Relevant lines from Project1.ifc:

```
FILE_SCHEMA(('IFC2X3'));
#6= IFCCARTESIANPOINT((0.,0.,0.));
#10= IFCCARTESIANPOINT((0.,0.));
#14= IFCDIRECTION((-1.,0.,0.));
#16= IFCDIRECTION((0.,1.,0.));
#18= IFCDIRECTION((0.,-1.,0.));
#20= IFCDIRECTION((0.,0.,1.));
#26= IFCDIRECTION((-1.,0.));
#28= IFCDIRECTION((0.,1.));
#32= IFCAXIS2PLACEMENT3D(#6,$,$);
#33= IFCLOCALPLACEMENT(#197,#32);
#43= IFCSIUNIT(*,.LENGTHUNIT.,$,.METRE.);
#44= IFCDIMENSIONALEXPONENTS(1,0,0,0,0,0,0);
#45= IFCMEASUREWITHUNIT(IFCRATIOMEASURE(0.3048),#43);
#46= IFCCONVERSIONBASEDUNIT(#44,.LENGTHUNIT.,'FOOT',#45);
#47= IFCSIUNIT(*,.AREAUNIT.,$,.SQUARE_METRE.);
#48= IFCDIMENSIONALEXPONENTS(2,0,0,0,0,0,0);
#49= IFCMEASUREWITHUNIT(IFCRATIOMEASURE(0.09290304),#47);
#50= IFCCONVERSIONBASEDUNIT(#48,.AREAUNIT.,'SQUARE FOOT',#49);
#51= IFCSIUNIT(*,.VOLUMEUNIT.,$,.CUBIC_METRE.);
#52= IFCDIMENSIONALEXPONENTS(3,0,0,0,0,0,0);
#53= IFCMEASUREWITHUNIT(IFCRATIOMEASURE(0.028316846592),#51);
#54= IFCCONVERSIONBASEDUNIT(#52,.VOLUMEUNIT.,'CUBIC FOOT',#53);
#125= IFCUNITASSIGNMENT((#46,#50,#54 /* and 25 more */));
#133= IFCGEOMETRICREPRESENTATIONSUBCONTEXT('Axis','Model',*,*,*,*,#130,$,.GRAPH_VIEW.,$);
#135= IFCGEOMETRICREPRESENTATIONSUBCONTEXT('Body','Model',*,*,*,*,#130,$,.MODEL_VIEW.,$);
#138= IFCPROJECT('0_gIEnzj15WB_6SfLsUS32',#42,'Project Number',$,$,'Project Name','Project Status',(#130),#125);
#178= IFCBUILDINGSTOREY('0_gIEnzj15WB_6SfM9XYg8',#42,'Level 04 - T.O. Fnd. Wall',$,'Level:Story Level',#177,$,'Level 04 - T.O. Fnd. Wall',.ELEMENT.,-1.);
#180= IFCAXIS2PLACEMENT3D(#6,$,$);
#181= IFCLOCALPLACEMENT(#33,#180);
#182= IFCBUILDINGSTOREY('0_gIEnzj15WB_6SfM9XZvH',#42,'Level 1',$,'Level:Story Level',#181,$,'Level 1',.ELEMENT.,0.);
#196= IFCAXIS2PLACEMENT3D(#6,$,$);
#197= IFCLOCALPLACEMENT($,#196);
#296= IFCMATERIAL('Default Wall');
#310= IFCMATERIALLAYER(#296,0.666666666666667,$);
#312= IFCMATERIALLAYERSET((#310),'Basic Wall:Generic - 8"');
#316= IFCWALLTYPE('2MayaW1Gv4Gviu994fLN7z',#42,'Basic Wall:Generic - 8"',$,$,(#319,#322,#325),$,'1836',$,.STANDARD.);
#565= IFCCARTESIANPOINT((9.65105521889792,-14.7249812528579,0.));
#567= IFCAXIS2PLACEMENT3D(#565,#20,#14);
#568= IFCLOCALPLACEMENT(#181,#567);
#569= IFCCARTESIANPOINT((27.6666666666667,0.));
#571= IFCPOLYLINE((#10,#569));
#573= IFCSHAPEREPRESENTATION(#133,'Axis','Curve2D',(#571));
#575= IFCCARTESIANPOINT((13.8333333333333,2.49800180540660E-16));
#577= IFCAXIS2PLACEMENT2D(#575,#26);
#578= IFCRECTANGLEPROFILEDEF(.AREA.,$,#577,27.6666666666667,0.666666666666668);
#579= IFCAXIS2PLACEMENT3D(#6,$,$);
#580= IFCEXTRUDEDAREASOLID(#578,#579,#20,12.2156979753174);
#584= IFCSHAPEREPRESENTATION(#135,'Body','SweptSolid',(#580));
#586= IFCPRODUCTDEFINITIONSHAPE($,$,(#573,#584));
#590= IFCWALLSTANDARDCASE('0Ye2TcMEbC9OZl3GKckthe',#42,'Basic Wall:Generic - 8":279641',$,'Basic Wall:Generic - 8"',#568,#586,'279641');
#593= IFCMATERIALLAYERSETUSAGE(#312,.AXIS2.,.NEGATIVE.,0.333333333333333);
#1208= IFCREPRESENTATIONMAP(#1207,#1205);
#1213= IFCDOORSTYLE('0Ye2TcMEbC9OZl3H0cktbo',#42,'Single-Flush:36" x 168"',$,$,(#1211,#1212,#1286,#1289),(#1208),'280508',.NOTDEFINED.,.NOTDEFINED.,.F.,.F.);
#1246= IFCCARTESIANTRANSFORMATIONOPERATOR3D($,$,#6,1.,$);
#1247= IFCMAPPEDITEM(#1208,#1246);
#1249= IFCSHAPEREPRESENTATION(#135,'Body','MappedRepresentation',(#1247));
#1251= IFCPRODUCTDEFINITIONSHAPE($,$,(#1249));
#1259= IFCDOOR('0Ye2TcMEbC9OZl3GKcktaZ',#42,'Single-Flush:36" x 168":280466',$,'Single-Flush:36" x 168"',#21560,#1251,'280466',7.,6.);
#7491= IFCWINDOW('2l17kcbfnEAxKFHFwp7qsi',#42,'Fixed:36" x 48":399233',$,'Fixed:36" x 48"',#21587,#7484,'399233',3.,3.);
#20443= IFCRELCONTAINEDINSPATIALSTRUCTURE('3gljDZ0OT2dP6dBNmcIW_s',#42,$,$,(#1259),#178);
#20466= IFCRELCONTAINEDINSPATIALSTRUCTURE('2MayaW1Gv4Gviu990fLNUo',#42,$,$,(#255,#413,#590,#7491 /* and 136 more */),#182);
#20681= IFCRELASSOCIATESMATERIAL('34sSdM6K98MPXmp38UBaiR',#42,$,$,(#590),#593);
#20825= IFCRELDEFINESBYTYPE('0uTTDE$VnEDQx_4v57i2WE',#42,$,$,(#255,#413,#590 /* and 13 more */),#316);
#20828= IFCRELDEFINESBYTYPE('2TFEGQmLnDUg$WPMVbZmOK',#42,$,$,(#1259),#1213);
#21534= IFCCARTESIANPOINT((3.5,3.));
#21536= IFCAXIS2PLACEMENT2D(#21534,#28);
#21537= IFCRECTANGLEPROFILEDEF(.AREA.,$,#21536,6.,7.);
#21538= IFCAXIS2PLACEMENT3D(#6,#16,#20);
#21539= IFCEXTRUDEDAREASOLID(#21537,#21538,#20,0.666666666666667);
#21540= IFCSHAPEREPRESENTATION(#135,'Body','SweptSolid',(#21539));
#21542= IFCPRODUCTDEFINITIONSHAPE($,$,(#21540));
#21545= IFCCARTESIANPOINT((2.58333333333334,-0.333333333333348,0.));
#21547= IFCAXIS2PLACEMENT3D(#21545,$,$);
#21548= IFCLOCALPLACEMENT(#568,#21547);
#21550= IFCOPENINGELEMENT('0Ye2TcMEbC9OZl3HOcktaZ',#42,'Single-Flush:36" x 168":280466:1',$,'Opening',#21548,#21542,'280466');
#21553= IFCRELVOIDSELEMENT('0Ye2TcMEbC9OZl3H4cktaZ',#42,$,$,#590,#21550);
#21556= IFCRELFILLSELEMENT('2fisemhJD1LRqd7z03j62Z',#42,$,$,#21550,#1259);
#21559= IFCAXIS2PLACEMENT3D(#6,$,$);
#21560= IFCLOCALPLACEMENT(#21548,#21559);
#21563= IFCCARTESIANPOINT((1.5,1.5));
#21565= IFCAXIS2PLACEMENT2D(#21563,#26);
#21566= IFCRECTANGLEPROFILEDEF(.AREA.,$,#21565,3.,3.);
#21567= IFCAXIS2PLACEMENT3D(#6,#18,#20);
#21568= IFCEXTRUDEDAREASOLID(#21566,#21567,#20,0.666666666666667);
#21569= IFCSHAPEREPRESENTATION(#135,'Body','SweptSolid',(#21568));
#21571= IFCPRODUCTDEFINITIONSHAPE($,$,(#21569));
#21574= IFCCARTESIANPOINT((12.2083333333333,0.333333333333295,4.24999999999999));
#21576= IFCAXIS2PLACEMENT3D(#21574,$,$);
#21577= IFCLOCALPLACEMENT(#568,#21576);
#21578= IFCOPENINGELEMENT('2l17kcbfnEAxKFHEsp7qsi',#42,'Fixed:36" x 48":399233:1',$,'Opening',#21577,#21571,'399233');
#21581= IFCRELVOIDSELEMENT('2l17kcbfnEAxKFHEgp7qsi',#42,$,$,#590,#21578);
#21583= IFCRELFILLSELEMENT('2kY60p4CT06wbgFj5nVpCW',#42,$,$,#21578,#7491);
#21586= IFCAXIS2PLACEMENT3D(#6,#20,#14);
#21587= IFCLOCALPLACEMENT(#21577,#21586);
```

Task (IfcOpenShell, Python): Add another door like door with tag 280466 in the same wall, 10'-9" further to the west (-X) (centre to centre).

```python
import ifcopenshell
import ifcopenshell.api.feature
import ifcopenshell.api.geometry
import ifcopenshell.api.root
import ifcopenshell.geom
import ifcopenshell.util.element
import ifcopenshell.util.placement
import ifcopenshell.util.shape
import ifcopenshell.util.unit

model = ifcopenshell.open("Project1.ifc")
unit_scale = ifcopenshell.util.unit.calculate_unit_scale(model)
settings = ifcopenshell.geom.settings()


def volume(element):
    """Net volume in cubic metres, openings subtracted."""
    shape = ifcopenshell.geom.create_shape(settings, element)
    return ifcopenshell.util.shape.get_volume(shape.geometry)


def reuse_history(source, copy):
    """copy_class also copies each property set's owner history, people and application; keep the originals."""
    for rel in copy.IsDefinedBy:
        if rel.is_a("IfcRelDefinesByProperties") and (history := rel.RelatingPropertyDefinition.OwnerHistory):
            rel.RelatingPropertyDefinition.OwnerHistory = source.OwnerHistory
            ifcopenshell.util.element.remove_deep2(model, history)


door = model.by_id(1259)
opening = door.FillsVoids[0].RelatingOpeningElement
wall = opening.VoidsElements[0].RelatingBuildingElement
before = volume(wall)
shift = ifcopenshell.util.placement.get_local_placement(wall.ObjectPlacement)[:3, 0] * 129 * 0.0254 / unit_scale

# copy_class copies the void relationship, type, container and properties, but no geometry.
new_opening = ifcopenshell.api.root.copy_class(model, product=opening)
new_opening.Representation = ifcopenshell.util.element.copy_deep(
    model, opening.Representation, exclude=["IfcGeometricRepresentationContext", "IfcRepresentationMap"]
)
new_opening.Name = 'Single-Flush:36" x 168"'
new_opening.Tag = None
new_door = ifcopenshell.api.root.copy_class(model, product=door)
new_door.Representation = ifcopenshell.util.element.copy_deep(
    model, door.Representation, exclude=["IfcGeometricRepresentationContext", "IfcRepresentationMap"]
)
new_door.Name = 'Single-Flush:36" x 168"'
new_door.Tag = None
reuse_history(door, new_door)
fills = ifcopenshell.api.feature.add_filling(model, opening=new_opening, element=new_door)
fills.OwnerHistory = new_door.OwnerHistory  # required in IFC2X3

for old, new in ((opening, new_opening), (door, new_door)):
    matrix = ifcopenshell.util.placement.get_local_placement(old.ObjectPlacement)
    matrix[:3, 3] += shift
    ifcopenshell.api.geometry.edit_object_placement(model, product=new, matrix=matrix, is_si=False)

after = volume(wall)

print(f"wall volume {before:.3f} -> {after:.3f} m3")

model.write("Project1-out.ifc")
```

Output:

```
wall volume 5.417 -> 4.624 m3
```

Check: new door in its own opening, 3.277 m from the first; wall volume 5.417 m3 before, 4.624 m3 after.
